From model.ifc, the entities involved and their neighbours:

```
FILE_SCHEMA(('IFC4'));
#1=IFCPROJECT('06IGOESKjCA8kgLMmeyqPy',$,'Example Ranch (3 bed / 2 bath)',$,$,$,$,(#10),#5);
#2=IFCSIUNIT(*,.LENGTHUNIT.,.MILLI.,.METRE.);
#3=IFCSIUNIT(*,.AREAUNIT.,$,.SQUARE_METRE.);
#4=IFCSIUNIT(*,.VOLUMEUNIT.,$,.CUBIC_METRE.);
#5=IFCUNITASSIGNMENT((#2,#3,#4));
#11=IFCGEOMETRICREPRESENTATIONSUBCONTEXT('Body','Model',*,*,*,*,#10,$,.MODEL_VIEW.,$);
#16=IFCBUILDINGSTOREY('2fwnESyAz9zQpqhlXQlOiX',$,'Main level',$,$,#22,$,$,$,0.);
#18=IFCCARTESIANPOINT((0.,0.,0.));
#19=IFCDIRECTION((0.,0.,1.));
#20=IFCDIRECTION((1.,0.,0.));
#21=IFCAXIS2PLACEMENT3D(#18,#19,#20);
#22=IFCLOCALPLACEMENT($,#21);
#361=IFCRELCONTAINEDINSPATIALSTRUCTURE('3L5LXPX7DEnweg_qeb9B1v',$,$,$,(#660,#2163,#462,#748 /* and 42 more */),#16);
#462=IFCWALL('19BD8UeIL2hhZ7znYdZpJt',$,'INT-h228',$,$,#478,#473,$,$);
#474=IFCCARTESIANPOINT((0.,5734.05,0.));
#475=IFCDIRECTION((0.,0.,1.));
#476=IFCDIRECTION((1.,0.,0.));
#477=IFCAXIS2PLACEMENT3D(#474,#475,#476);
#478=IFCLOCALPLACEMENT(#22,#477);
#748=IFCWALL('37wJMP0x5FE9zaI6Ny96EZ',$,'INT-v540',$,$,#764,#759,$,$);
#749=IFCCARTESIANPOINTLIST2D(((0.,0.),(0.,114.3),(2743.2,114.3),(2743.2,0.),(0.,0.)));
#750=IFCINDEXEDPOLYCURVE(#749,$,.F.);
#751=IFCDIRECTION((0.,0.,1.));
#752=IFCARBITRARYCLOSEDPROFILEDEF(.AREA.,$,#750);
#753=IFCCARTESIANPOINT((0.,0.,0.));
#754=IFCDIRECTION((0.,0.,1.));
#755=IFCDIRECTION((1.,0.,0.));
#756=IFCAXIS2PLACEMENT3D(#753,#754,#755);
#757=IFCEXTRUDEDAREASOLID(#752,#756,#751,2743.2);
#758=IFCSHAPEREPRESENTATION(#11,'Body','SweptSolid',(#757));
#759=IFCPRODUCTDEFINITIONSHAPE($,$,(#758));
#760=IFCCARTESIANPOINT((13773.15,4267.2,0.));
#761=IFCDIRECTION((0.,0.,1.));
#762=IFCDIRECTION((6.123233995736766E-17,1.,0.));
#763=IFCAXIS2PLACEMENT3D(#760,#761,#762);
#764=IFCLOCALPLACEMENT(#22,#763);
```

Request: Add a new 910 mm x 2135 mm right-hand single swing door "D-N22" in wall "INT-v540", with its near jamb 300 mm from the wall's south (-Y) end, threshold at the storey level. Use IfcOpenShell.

```python
import numpy as np
import ifcopenshell
import ifcopenshell.api.feature
import ifcopenshell.api.geometry
import ifcopenshell.api.root
import ifcopenshell.api.spatial
import ifcopenshell.geom
import ifcopenshell.util.element
import ifcopenshell.util.placement
import ifcopenshell.util.representation
import ifcopenshell.util.shape
import ifcopenshell.util.unit

model = ifcopenshell.open("model.ifc")
unit_scale = ifcopenshell.util.unit.calculate_unit_scale(model)
settings = ifcopenshell.geom.settings()


def volume(element):
    """Net volume in cubic metres, openings subtracted."""
    shape = ifcopenshell.geom.create_shape(settings, element)
    return ifcopenshell.util.shape.get_volume(shape.geometry)


wall = model.by_guid("37wJMP0x5FE9zaI6Ny96EZ")
storey = ifcopenshell.util.element.get_container(wall, ifc_class="IfcBuildingStorey")
context = ifcopenshell.util.representation.get_context(model, "Model", "Body", "MODEL_VIEW")
before = volume(wall)

width, height, from_end, sill = 0.91, 2.135, 0.3, 0.0  # metres

# The wall runs along its own X axis, and the end named is its -X end.
wall_shape = ifcopenshell.geom.create_shape(settings, wall)
x, y, z = ifcopenshell.util.shape.get_vertices(wall_shape.geometry).T
start = x.min() + from_end
face, thickness = float(y.min()), float(y.max() - y.min())
wall_matrix = ifcopenshell.util.placement.get_local_placement(wall.ObjectPlacement)
level = ifcopenshell.util.placement.get_local_placement(storey.ObjectPlacement)[2, 3]


def in_wall(x, y):
    """Placement at x, y metres in the wall's axes, at sill height."""
    matrix = wall_matrix.copy()
    matrix[:, 3] = wall_matrix @ np.array([x / unit_scale, y / unit_scale, 0.0, 1.0])
    matrix[2, 3] = level + sill / unit_scale
    return matrix


# Opening: a box that overshoots both wall faces by 50 mm.
opening = ifcopenshell.api.root.create_entity(model, ifc_class="IfcOpeningElement", predefined_type="OPENING")
box = ifcopenshell.api.geometry.add_wall_representation(
    model, context=context, length=width, height=height, thickness=thickness + 0.1
)
ifcopenshell.api.geometry.assign_representation(model, product=opening, representation=box)
ifcopenshell.api.geometry.edit_object_placement(model, product=opening, matrix=in_wall(start, face - 0.05), is_si=False)
ifcopenshell.api.feature.add_feature(model, feature=opening, element=wall)

door = ifcopenshell.api.root.create_entity(model, ifc_class="IfcDoor", name="D-N22", predefined_type="DOOR")
door.OverallWidth, door.OverallHeight = width / unit_scale, height / unit_scale
door.OperationType = "SINGLE_SWING_RIGHT"
body = ifcopenshell.api.geometry.add_door_representation(
    model,
    context=context,
    overall_width=door.OverallWidth,
    overall_height=door.OverallHeight,
    operation_type="SINGLE_SWING_RIGHT",
    lining_properties={"LiningDepth": thickness / unit_scale, "ThresholdDepth": thickness / unit_scale},
)
ifcopenshell.api.geometry.assign_representation(model, product=door, representation=body)
ifcopenshell.api.spatial.assign_container(model, products=[door], relating_structure=storey)
ifcopenshell.api.feature.add_filling(model, opening=opening, element=door)

# The lining spans the wall, so the door starts at the wall face.
ifcopenshell.api.geometry.edit_object_placement(model, product=door, matrix=in_wall(start, face), is_si=False)

after = volume(wall)

print(f"wall volume {before:.3f} -> {after:.3f} m3")

model.write("model_updated.ifc")
```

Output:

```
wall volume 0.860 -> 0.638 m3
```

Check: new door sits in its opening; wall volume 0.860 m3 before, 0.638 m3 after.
